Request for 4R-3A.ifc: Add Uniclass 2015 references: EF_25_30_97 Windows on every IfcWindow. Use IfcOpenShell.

First a look at what the model holds.

```python
import ifcopenshell

model = ifcopenshell.open("4R-3A.ifc")
print(model.schema)
print("classifications:", [c.Name for c in model.by_type("IfcClassification")])
for ifc_class in ("IfcDoor", "IfcRoof", "IfcStair", "IfcWall", "IfcWindow"):
    print(ifc_class, len(model.by_type(ifc_class)))
```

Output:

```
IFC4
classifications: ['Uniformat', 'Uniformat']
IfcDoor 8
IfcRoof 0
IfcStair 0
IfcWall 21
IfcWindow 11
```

```python
import ifcopenshell
import ifcopenshell.api.classification

model = ifcopenshell.open("4R-3A.ifc")

system = ifcopenshell.api.classification.add_classification(model, classification="Uniclass 2015")

codes = {
    "IfcWindow": ("EF_25_30_97", "Windows"),
}
for ifc_class, (code, name) in codes.items():
    products = model.by_type(ifc_class)
    ifcopenshell.api.classification.add_reference(
        model, products=products, classification=system, identification=code, name=name
    )
    print(code, len(products))

model.write("4R-3A_updated.ifc")
```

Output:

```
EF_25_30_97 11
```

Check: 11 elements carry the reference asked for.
